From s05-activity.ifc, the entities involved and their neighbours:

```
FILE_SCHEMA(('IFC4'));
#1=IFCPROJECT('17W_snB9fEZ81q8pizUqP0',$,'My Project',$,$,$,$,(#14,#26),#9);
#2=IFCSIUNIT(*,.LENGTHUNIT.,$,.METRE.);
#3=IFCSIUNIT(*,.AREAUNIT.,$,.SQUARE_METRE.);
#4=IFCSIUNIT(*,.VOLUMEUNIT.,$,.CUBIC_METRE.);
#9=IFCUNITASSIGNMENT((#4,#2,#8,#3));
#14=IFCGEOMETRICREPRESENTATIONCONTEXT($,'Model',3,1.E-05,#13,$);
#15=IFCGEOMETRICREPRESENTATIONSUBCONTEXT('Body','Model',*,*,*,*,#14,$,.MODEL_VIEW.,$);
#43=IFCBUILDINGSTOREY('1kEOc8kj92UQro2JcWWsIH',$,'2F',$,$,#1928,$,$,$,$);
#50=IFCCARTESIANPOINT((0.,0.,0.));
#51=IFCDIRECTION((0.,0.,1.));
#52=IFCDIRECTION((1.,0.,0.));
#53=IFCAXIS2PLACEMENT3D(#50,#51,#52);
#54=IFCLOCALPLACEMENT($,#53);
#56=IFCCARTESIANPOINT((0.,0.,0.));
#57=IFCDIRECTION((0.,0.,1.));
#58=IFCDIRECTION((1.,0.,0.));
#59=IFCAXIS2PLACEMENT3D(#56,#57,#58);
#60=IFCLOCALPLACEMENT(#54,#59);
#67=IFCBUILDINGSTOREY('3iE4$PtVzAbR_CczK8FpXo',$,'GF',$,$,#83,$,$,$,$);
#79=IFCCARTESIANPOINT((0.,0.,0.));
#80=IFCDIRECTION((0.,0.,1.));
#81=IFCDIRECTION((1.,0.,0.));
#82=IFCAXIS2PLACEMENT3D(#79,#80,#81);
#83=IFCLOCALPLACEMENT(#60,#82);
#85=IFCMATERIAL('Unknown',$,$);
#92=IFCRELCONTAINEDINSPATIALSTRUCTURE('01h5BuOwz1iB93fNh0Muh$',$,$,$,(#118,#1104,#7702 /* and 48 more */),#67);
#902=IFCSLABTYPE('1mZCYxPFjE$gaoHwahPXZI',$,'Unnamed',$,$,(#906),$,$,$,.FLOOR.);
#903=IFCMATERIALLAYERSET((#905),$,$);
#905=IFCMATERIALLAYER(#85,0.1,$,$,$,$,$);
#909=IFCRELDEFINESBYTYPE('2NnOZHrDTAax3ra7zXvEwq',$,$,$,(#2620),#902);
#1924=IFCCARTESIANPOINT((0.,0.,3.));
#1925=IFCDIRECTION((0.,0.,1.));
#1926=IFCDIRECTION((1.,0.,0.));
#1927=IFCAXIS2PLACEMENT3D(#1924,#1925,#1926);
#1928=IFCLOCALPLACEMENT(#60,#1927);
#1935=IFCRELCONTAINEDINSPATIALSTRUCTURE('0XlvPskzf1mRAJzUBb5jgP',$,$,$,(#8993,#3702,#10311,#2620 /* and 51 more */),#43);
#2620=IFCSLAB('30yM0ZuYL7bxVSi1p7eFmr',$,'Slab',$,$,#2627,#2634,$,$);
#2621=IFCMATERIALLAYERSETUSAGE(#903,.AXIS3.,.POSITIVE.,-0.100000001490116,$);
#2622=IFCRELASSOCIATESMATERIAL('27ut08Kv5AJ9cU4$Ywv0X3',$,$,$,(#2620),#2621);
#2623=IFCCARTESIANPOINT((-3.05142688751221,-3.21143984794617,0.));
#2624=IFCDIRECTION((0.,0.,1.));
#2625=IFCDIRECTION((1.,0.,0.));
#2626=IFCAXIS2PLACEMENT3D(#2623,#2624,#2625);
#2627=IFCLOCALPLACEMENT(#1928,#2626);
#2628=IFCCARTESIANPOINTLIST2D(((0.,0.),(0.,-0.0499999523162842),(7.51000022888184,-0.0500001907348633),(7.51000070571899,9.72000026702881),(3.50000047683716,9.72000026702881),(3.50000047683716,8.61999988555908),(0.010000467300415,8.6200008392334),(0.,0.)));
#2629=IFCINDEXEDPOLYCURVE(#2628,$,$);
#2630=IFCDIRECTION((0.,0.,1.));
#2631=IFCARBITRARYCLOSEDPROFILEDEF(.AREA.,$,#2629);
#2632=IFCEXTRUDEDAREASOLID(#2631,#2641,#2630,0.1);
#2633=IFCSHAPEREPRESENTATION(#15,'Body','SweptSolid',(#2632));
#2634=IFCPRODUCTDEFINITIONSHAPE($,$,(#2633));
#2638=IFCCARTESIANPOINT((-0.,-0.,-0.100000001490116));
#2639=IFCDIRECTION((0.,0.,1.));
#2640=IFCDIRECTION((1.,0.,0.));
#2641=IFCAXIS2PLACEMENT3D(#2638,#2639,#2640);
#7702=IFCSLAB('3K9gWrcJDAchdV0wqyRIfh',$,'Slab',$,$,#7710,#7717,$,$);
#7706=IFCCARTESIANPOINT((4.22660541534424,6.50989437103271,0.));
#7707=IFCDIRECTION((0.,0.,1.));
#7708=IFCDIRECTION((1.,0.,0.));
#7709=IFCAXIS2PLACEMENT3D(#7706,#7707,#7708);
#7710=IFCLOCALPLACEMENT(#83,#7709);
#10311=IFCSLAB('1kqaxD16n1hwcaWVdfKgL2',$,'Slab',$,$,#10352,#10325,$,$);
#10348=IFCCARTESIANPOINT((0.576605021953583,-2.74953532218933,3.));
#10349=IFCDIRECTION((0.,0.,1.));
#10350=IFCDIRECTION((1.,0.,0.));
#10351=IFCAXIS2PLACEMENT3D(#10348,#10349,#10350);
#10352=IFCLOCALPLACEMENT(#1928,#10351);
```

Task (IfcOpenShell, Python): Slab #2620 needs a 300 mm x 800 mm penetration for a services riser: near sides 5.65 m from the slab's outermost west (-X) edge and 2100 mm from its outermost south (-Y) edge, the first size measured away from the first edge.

```python
import numpy as np
import ifcopenshell
import ifcopenshell.api.feature
import ifcopenshell.api.geometry
import ifcopenshell.api.root
import ifcopenshell.geom
import ifcopenshell.util.placement
import ifcopenshell.util.representation
import ifcopenshell.util.shape
import ifcopenshell.util.unit

model = ifcopenshell.open("s05-activity.ifc")
unit_scale = ifcopenshell.util.unit.calculate_unit_scale(model)
settings = ifcopenshell.geom.settings()


def volume(element):
    """Net volume in cubic metres, openings subtracted."""
    shape = ifcopenshell.geom.create_shape(settings, element)
    return ifcopenshell.util.shape.get_volume(shape.geometry)


slab = model.by_guid("30yM0ZuYL7bxVSi1p7eFmr")
before = volume(slab)

# Extent in the slab's own axes, in metres. The edges named are its -X and -Y sides.
slab_shape = ifcopenshell.geom.create_shape(settings, slab)
vertices = ifcopenshell.util.shape.get_vertices(slab_shape.geometry)
x_min, y_min, bottom = vertices.min(axis=0)
top = vertices[:, 2].max()

opening = ifcopenshell.api.root.create_entity(model, ifc_class="IfcOpeningElement", name="Services riser opening", predefined_type="OPENING")
context = ifcopenshell.util.representation.get_context(model, "Model", "Body", "MODEL_VIEW")
width, depth = 0.3, 0.8
outline = [(0.0, 0.0), (width, 0.0), (width, depth), (0.0, depth), (0.0, 0.0)]
# Overshoot both faces by 50 mm so the cut is clean.
shape = ifcopenshell.api.geometry.add_slab_representation(
    model, context=context, depth=top - bottom + 0.1, polyline=outline
)
ifcopenshell.api.geometry.assign_representation(model, product=opening, representation=shape)

matrix = ifcopenshell.util.placement.get_local_placement(slab.ObjectPlacement)
matrix[:, 3] = matrix @ np.append(np.array([x_min + 5.65, y_min + 2.1, bottom - 0.05]) / unit_scale, 1.0)
ifcopenshell.api.geometry.edit_object_placement(model, product=opening, matrix=matrix, is_si=False)
ifcopenshell.api.feature.add_feature(model, feature=opening, element=slab)

after = volume(slab)

print(f"slab volume {before:.3f} -> {after:.3f} m3")

model.write("s05-activity_updated.ifc")
```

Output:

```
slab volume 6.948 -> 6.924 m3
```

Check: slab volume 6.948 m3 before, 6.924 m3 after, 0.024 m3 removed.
